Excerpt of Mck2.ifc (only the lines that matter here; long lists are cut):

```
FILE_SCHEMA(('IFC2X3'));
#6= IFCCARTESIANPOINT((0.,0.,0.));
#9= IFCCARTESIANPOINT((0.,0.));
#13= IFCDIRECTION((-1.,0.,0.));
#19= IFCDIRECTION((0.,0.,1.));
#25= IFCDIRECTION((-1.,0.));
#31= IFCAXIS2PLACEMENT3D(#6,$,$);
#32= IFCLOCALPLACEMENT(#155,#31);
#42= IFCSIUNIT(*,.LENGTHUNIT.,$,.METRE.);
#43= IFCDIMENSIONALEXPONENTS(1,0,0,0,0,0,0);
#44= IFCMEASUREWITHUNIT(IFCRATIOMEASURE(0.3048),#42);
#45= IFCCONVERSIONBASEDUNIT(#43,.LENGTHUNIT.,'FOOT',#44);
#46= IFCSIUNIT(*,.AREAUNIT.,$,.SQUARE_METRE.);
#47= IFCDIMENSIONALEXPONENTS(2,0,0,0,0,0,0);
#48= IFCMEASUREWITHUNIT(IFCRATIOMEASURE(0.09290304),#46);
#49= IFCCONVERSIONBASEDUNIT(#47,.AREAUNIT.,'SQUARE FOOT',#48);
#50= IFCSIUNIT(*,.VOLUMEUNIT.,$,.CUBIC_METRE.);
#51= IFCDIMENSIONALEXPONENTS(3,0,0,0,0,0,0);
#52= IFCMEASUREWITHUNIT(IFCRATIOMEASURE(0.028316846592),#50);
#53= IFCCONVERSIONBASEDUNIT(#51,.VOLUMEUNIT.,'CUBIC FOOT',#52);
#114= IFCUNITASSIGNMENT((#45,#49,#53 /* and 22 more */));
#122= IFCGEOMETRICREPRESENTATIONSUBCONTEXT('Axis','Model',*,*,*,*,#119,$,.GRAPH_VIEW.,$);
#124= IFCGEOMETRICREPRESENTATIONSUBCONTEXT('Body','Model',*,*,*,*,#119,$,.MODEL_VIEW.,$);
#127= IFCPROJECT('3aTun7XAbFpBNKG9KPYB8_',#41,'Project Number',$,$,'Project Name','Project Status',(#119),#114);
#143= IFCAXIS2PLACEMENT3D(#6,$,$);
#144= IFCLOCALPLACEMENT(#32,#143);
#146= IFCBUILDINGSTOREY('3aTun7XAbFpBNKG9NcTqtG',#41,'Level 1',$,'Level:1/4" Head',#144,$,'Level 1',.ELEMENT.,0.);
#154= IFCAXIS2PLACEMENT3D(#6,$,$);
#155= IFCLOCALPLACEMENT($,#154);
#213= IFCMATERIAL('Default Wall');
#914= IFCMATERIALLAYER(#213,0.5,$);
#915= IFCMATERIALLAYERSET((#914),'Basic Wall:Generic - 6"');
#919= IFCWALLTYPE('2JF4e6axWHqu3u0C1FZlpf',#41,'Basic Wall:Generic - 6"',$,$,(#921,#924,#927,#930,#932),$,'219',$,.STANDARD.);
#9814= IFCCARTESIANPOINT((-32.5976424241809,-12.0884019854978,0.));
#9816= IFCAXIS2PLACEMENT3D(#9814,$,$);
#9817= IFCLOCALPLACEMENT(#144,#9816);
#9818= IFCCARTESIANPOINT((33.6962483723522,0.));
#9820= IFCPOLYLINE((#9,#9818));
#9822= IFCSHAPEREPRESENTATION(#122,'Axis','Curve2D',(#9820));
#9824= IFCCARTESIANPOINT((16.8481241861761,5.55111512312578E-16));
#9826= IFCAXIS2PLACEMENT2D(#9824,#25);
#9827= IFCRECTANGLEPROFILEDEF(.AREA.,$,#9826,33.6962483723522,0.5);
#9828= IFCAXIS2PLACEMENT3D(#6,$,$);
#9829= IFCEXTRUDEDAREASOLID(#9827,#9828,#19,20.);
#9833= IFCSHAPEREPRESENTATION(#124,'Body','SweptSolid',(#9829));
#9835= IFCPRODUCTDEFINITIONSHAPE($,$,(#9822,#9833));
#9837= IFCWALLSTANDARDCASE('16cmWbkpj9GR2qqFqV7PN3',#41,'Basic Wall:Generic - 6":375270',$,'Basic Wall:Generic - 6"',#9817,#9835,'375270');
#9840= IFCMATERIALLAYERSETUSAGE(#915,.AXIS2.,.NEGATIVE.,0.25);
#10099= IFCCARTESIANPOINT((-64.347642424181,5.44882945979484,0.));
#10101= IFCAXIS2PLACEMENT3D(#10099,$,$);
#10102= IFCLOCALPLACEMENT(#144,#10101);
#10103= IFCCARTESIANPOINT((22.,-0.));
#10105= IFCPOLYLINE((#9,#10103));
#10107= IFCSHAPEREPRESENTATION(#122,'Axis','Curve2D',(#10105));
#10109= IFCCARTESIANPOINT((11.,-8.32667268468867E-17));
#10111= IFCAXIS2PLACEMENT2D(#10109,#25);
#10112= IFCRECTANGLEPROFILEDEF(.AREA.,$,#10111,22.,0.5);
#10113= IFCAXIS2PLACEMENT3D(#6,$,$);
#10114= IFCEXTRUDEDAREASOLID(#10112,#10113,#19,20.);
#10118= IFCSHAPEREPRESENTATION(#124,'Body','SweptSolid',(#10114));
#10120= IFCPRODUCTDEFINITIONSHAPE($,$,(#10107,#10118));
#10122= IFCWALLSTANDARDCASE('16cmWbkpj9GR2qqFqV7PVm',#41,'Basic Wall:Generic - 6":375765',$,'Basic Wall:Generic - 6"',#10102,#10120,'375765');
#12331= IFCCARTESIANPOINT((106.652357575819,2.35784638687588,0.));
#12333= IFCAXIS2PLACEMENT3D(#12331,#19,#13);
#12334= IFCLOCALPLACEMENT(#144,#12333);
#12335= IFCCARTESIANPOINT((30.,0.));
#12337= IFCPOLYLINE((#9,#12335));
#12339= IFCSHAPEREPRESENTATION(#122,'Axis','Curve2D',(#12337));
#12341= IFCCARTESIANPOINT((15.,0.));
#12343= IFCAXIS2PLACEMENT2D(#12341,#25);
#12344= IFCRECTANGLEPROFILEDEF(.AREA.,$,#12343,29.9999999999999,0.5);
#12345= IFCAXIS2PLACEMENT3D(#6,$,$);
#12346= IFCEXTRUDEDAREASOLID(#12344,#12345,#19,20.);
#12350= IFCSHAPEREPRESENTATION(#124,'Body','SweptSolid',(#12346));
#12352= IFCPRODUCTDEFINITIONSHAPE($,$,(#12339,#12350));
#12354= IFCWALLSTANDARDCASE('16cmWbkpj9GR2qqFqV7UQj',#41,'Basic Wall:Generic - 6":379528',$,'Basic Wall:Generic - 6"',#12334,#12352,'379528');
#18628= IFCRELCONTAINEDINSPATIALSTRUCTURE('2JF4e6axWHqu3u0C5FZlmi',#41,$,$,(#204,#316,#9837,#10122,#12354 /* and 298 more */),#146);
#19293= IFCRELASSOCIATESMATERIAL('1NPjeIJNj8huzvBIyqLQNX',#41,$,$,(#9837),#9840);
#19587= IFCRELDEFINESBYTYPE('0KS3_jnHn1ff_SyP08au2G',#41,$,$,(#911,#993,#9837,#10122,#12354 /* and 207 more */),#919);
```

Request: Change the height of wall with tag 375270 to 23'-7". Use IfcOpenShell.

```python
import ifcopenshell
import ifcopenshell.geom
import ifcopenshell.util.representation
import ifcopenshell.util.shape
import ifcopenshell.util.unit

model = ifcopenshell.open("Mck2.ifc")
unit_scale = ifcopenshell.util.unit.calculate_unit_scale(model)
settings = ifcopenshell.geom.settings()


def volume(element):
    """Net volume in cubic metres, openings subtracted."""
    shape = ifcopenshell.geom.create_shape(settings, element)
    return ifcopenshell.util.shape.get_volume(shape.geometry)


wall = model.by_id(9837)
before = volume(wall)

body = ifcopenshell.util.representation.get_representation(wall, "Model", "Body")
solid = body.Items[0]
old_height = solid.Depth
solid.Depth = 283 * 0.0254 / unit_scale
after = volume(wall)

print(f"height {old_height:g} -> {solid.Depth:g}, volume {before:.3f} -> {after:.3f} m3")

model.write("Mck2_v2.ifc")
```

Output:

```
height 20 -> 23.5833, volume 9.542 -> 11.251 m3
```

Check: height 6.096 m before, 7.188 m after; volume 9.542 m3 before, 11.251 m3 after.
